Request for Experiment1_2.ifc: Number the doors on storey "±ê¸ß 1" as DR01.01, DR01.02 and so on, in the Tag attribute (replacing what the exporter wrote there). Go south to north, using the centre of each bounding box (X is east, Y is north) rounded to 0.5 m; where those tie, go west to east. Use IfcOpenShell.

First a look at what the model holds.

```python
import ifcopenshell
import ifcopenshell.util.element
import ifcopenshell.util.placement

model = ifcopenshell.open("Experiment1_2.ifc")
print(model.schema)
storey = next(s for s in model.by_type("IfcBuildingStorey") if s.Name == "±ê¸ß 1")
doors = [e for e in ifcopenshell.util.element.get_decomposition(storey) if e.is_a("IfcDoor")]
for e in sorted(doors, key=lambda e: e.id()):
    origin = ifcopenshell.util.placement.get_local_placement(e.ObjectPlacement)[:3, 3]
    print(e.id(), e.Tag, e.Name, origin.round(2) + 0.0, sep=" | ")
```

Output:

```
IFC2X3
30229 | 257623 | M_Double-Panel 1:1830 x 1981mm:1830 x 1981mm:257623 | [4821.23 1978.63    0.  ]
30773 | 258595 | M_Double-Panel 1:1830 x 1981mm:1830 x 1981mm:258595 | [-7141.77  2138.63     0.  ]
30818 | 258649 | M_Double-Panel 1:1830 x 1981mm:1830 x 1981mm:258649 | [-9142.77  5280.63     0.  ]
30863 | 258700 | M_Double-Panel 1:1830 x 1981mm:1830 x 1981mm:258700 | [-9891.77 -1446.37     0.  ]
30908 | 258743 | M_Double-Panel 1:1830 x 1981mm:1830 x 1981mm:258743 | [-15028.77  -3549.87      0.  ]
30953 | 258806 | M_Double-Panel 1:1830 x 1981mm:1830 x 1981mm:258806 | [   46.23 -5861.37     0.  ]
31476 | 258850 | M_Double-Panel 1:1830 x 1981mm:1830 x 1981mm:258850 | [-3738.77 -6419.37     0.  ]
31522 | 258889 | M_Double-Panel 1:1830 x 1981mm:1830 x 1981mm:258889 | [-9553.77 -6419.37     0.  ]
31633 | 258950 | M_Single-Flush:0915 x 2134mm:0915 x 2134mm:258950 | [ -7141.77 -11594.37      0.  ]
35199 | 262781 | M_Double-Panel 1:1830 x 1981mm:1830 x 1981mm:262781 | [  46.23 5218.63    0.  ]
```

```python
import ifcopenshell
import ifcopenshell.geom
import ifcopenshell.util.element
import ifcopenshell.util.shape

model = ifcopenshell.open("Experiment1_2.ifc")
settings = ifcopenshell.geom.settings()
settings.set("use-world-coords", True)


def centre(element):
    shape = ifcopenshell.geom.create_shape(settings, element)
    return ifcopenshell.util.shape.get_bbox_centroid(shape.geometry)


storey = next(s for s in model.by_type("IfcBuildingStorey") if s.Name == "±ê¸ß 1")
doors = [e for e in ifcopenshell.util.element.get_decomposition(storey) if e.is_a("IfcDoor")]

# Insertion points can sit at a corner or the storey origin, so sort by the geometry (in metres).
centres = {e: centre(e) for e in doors}
doors.sort(key=lambda e: (round(centres[e][1] / 0.5), centres[e][0]))

for i, e in enumerate(doors, start=1):
    number = f"DR01.{i:02d}"
    e.Tag = number
    print(e.id(), number)

model.write("Experiment1_2-out.ifc")
```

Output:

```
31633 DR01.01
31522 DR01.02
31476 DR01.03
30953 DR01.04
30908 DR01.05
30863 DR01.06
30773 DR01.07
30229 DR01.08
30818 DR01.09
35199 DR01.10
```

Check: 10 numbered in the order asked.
